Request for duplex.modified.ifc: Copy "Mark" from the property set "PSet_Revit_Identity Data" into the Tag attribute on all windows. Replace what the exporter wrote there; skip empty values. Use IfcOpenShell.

First a look at what the model holds.

```python
import ifcopenshell
import ifcopenshell.util.element

model = ifcopenshell.open("duplex.modified.ifc")
print(model.schema)
windows = model.by_type("IfcWindow")
print(len(windows), "windows")
for e in windows[:8]:
    source = ifcopenshell.util.element.get_pset(e, "PSet_Revit_Identity Data", "Mark")
    target = e.Tag
    print(e.id(), repr(source), repr(target), sep=" | ")
```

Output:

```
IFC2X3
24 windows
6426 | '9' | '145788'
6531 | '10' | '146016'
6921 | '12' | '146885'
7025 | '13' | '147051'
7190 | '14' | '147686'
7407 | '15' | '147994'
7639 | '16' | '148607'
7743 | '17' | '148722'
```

```python
import ifcopenshell
import ifcopenshell.util.element

model = ifcopenshell.open("duplex.modified.ifc")

count = 0
for e in model.by_type("IfcWindow"):
    value = ifcopenshell.util.element.get_pset(e, "PSet_Revit_Identity Data", "Mark")
    current = e.Tag
    if not value or not value.strip() or current == value:
        continue
    e.Tag = value
    count += 1

print(count, "windows updated")

model.write("duplex.modified_rev.ifc")
```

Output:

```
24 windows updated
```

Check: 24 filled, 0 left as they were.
